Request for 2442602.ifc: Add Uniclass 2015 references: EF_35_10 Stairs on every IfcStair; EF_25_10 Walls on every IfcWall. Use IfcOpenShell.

First a look at what the model holds.

```python
import ifcopenshell

model = ifcopenshell.open("2442602.ifc")
print(model.schema)
print("classifications:", [c.Name for c in model.by_type("IfcClassification")])
for ifc_class in ("IfcDoor", "IfcRoof", "IfcStair", "IfcWall", "IfcWindow"):
    print(ifc_class, len(model.by_type(ifc_class)))
```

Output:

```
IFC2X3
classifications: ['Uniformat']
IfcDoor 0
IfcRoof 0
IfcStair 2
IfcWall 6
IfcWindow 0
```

```python
import ifcopenshell
import ifcopenshell.api.classification

model = ifcopenshell.open("2442602.ifc")

# IFC2X3 requires Source and Edition and has no link from the project to the system.
system = model.create_entity("IfcClassification", Source="NBS", Edition="2015", Name="Uniclass 2015")

codes = {
    "IfcStair": ("EF_35_10", "Stairs"),
    "IfcWall": ("EF_25_10", "Walls"),
}
for ifc_class, (code, name) in codes.items():
    products = model.by_type(ifc_class)
    ifcopenshell.api.classification.add_reference(
        model, products=products, classification=system, identification=code, name=name
    )
    print(code, len(products))

model.write("2442602-out.ifc")
```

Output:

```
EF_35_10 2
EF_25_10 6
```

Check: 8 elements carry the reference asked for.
